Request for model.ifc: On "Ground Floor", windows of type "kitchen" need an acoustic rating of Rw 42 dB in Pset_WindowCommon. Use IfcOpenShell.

First a look at what the model holds.

```python
import ifcopenshell
import ifcopenshell.util.element

model = ifcopenshell.open("model.ifc")
print(model.schema)
storey = next(s for s in model.by_type("IfcBuildingStorey") if s.Name == "Ground Floor")
windows = [e for e in ifcopenshell.util.element.get_decomposition(storey) if e.is_a("IfcWindow")]
seen = {}
for e in windows:
    element_type = ifcopenshell.util.element.get_type(e)
    key = (element_type.Name if element_type != e and element_type else None, ifcopenshell.util.element.get_pset(e, "Pset_WindowCommon", "AcousticRating"))
    seen[key] = seen.get(key, 0) + 1
for (name, value), count in sorted(seen.items(), key=str):
    print(count, "x", name, "|", value)
```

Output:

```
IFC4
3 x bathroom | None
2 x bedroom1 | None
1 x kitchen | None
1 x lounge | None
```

```python
import ifcopenshell
import ifcopenshell.api.pset
import ifcopenshell.util.element

model = ifcopenshell.open("model.ifc")

storey = next(s for s in model.by_type("IfcBuildingStorey") if s.Name == "Ground Floor")
windows = [e for e in ifcopenshell.util.element.get_decomposition(storey) if e.is_a("IfcWindow")]

count = 0
for e in windows:
    element_type = ifcopenshell.util.element.get_type(e)
    if element_type in (None, e) or element_type.Name != "kitchen":
        continue
    # add_pset returns the element's existing set when there is one.
    pset = ifcopenshell.api.pset.add_pset(model, product=e, name="Pset_WindowCommon")
    ifcopenshell.api.pset.edit_pset(model, pset=pset, properties={"AcousticRating": "Rw 42 dB"})
    count += 1

print(count, "windows updated")

model.write("model_updated.ifc")
```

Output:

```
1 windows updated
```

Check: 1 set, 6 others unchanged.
